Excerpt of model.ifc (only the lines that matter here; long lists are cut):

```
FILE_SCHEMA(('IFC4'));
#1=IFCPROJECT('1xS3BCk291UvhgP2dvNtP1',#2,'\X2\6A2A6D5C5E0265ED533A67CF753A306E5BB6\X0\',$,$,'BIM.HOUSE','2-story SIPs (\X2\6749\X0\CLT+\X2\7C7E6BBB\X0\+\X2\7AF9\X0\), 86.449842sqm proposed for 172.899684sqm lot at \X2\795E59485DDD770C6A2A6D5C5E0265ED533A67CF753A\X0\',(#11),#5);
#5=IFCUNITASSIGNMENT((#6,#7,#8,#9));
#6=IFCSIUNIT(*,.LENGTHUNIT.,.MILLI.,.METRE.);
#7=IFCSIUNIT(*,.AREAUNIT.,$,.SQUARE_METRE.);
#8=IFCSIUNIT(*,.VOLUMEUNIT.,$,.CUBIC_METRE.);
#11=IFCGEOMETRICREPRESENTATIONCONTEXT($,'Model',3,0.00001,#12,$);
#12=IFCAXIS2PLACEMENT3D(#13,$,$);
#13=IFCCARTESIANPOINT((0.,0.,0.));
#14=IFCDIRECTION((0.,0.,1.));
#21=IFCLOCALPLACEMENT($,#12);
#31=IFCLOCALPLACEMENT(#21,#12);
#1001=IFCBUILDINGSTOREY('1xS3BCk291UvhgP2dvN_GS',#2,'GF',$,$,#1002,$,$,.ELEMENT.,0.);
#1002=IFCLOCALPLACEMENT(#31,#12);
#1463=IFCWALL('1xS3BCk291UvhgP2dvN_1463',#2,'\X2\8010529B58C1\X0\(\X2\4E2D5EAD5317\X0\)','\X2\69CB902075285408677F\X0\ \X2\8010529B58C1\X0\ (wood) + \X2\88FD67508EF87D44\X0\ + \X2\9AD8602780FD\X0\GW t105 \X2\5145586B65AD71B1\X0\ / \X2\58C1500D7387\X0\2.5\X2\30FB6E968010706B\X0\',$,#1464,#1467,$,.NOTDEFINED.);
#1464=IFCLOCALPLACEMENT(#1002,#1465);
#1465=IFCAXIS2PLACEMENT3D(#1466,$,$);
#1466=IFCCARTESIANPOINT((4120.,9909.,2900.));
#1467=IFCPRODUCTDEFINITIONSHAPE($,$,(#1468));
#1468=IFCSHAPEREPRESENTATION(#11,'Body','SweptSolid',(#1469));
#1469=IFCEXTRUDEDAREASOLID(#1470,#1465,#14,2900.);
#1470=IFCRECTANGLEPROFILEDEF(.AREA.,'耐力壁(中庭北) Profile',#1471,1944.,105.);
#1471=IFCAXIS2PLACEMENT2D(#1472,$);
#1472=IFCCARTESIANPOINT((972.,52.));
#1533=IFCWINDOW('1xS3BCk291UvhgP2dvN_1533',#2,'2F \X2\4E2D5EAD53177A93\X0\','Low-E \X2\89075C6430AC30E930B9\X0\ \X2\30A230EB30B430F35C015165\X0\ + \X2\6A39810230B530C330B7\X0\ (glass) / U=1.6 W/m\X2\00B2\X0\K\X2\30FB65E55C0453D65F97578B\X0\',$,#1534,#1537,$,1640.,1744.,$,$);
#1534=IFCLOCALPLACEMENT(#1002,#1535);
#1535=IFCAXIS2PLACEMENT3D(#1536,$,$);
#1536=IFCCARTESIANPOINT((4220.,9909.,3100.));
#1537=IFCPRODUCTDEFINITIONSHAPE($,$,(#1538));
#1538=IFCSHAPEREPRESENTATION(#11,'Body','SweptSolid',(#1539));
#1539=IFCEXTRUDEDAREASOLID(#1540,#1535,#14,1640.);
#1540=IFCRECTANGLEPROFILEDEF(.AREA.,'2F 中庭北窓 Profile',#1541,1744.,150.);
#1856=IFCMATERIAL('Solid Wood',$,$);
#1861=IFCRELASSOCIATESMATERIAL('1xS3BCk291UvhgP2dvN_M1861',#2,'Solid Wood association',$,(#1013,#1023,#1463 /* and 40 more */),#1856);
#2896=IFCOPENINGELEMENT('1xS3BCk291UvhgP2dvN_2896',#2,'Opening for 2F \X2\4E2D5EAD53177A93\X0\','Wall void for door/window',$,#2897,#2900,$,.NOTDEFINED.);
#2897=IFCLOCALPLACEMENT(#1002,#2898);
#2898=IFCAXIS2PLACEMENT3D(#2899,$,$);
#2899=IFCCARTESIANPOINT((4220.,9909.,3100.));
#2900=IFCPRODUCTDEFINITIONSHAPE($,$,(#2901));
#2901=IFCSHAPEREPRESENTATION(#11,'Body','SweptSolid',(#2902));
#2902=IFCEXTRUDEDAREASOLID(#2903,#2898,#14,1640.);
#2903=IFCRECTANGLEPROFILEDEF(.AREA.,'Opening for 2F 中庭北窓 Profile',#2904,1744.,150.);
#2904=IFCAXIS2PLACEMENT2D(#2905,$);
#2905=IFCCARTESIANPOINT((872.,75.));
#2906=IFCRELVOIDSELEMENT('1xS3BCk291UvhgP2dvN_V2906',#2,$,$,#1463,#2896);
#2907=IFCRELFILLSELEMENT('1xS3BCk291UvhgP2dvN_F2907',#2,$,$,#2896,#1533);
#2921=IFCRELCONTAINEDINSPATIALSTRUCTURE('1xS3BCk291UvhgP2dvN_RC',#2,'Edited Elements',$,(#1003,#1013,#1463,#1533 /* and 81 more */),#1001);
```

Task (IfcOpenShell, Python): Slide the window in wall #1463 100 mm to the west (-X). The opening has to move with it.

```python
import ifcopenshell
import ifcopenshell.api.geometry
import ifcopenshell.util.placement

model = ifcopenshell.open("model.ifc")

window = model.by_guid("1xS3BCk291UvhgP2dvN_1533")
opening = window.FillsVoids[0].RelatingOpeningElement
wall = opening.VoidsElements[0].RelatingBuildingElement

wall_matrix = ifcopenshell.util.placement.get_local_placement(wall.ObjectPlacement)
shift = wall_matrix[:3, 0] * -100.0
before = ifcopenshell.util.placement.get_local_placement(window.ObjectPlacement)[:3, 3].copy()

# The window is not placed relative to its opening, so move both.
for product in (opening, window):
    matrix = ifcopenshell.util.placement.get_local_placement(product.ObjectPlacement)
    matrix[:3, 3] += shift
    ifcopenshell.api.geometry.edit_object_placement(model, product=product, matrix=matrix, is_si=False)

after = ifcopenshell.util.placement.get_local_placement(window.ObjectPlacement)[:3, 3]
print("window moved by", (after - before).round(3) + 0.0)

model.write("model_v2.ifc")
```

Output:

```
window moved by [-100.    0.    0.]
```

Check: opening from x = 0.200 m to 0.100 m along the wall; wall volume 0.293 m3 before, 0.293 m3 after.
